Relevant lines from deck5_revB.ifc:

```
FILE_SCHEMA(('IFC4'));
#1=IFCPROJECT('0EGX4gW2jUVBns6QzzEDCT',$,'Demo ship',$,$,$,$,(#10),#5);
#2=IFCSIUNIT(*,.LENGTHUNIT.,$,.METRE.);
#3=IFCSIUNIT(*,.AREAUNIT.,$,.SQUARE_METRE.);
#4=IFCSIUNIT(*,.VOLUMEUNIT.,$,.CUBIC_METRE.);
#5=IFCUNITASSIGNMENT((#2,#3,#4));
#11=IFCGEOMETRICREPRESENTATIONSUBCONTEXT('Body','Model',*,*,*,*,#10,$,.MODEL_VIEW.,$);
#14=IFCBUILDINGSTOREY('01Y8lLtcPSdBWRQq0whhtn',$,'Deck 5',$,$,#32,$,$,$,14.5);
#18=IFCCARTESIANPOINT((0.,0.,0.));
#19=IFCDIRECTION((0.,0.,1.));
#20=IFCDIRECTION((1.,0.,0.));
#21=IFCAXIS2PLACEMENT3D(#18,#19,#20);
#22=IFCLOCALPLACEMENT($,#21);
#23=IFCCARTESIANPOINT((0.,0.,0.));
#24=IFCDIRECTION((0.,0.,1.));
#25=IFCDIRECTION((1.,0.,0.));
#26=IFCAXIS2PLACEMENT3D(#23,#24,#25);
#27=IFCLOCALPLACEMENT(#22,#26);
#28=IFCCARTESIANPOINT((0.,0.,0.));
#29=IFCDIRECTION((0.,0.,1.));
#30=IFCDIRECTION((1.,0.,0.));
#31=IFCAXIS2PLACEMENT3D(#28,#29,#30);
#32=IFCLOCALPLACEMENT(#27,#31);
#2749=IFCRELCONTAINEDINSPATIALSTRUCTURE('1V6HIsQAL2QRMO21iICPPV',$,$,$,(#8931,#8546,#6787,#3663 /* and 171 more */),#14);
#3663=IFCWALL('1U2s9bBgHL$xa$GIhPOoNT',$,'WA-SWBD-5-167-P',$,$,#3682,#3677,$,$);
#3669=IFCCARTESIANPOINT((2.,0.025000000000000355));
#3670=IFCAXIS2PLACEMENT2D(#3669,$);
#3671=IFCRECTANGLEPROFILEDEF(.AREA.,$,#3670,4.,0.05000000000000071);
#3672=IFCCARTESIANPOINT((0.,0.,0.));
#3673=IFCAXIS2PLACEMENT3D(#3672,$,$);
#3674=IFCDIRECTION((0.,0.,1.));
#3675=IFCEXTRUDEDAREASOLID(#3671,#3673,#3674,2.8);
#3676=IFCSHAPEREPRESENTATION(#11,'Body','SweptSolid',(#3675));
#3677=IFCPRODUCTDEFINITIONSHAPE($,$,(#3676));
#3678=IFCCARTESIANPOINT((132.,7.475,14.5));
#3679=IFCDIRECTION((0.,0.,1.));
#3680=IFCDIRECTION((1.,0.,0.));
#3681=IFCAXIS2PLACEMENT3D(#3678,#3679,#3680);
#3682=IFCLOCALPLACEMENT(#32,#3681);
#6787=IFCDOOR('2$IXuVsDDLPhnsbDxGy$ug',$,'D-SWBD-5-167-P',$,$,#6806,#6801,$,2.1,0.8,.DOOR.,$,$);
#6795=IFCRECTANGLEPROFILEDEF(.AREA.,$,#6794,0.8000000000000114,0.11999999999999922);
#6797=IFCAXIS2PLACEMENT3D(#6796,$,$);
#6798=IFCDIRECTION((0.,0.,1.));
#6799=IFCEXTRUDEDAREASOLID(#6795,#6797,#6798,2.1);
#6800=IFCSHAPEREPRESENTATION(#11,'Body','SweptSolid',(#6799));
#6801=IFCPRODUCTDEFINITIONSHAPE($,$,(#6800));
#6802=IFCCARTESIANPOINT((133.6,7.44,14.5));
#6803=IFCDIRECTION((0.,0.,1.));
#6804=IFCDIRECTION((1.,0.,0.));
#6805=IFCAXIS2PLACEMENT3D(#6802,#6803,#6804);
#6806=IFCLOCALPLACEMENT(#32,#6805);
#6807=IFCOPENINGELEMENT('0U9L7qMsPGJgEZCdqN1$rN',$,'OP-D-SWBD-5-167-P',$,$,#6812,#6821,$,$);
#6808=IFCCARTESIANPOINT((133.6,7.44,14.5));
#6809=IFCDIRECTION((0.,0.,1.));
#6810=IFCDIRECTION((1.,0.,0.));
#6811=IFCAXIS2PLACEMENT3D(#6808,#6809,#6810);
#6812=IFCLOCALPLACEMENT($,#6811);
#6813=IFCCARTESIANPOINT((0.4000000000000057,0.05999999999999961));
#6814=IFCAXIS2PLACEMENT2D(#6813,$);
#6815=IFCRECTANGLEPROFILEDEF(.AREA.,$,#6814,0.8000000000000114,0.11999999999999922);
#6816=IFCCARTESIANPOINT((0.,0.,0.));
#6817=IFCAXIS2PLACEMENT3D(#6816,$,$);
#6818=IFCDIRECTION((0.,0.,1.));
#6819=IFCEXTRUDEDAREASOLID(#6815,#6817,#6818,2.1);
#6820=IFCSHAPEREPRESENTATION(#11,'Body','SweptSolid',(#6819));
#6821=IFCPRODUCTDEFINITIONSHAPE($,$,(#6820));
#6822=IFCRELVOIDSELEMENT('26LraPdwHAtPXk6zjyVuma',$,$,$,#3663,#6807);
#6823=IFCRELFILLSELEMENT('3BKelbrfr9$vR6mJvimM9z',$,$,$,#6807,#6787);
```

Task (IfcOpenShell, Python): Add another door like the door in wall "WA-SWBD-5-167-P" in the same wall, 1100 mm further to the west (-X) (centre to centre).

```python
import ifcopenshell
import ifcopenshell.api.feature
import ifcopenshell.api.geometry
import ifcopenshell.api.root
import ifcopenshell.geom
import ifcopenshell.util.element
import ifcopenshell.util.placement
import ifcopenshell.util.shape

model = ifcopenshell.open("deck5_revB.ifc")
settings = ifcopenshell.geom.settings()


def volume(element):
    """Net volume in cubic metres, openings subtracted."""
    shape = ifcopenshell.geom.create_shape(settings, element)
    return ifcopenshell.util.shape.get_volume(shape.geometry)


door = model.by_id(6787)
opening = door.FillsVoids[0].RelatingOpeningElement
wall = opening.VoidsElements[0].RelatingBuildingElement
before = volume(wall)
shift = ifcopenshell.util.placement.get_local_placement(wall.ObjectPlacement)[:3, 0] * -1.1

# copy_class copies the void relationship, type, container and properties, but no geometry.
new_opening = ifcopenshell.api.root.copy_class(model, product=opening)
new_opening.Representation = ifcopenshell.util.element.copy_deep(
    model, opening.Representation, exclude=["IfcGeometricRepresentationContext", "IfcRepresentationMap"]
)
new_door = ifcopenshell.api.root.copy_class(model, product=door)
new_door.Representation = ifcopenshell.util.element.copy_deep(
    model, door.Representation, exclude=["IfcGeometricRepresentationContext", "IfcRepresentationMap"]
)
ifcopenshell.api.feature.add_filling(model, opening=new_opening, element=new_door)

for old, new in ((opening, new_opening), (door, new_door)):
    matrix = ifcopenshell.util.placement.get_local_placement(old.ObjectPlacement)
    matrix[:3, 3] += shift
    ifcopenshell.api.geometry.edit_object_placement(model, product=new, matrix=matrix, is_si=False)

after = volume(wall)

print(f"wall volume {before:.3f} -> {after:.3f} m3")

model.write("deck5_revB-out.ifc")
```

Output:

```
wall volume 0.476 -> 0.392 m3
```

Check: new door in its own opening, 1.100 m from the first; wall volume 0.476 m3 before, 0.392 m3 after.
